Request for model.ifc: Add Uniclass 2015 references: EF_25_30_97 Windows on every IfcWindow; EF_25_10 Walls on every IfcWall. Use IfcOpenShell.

First a look at what the model holds.

```python
import ifcopenshell

model = ifcopenshell.open("model.ifc")
print(model.schema)
print("classifications:", [c.Name for c in model.by_type("IfcClassification")])
for ifc_class in ("IfcDoor", "IfcRoof", "IfcStair", "IfcWall", "IfcWindow"):
    print(ifc_class, len(model.by_type(ifc_class)))
```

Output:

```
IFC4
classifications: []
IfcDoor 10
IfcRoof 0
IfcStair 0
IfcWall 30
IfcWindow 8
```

```python
import ifcopenshell
import ifcopenshell.api.classification

model = ifcopenshell.open("model.ifc")

system = ifcopenshell.api.classification.add_classification(model, classification="Uniclass 2015")

codes = {
    "IfcWindow": ("EF_25_30_97", "Windows"),
    "IfcWall": ("EF_25_10", "Walls"),
}
for ifc_class, (code, name) in codes.items():
    products = model.by_type(ifc_class)
    ifcopenshell.api.classification.add_reference(
        model, products=products, classification=system, identification=code, name=name
    )
    print(code, len(products))

model.write("model_v2.ifc")
```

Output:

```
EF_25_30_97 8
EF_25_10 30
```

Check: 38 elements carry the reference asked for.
